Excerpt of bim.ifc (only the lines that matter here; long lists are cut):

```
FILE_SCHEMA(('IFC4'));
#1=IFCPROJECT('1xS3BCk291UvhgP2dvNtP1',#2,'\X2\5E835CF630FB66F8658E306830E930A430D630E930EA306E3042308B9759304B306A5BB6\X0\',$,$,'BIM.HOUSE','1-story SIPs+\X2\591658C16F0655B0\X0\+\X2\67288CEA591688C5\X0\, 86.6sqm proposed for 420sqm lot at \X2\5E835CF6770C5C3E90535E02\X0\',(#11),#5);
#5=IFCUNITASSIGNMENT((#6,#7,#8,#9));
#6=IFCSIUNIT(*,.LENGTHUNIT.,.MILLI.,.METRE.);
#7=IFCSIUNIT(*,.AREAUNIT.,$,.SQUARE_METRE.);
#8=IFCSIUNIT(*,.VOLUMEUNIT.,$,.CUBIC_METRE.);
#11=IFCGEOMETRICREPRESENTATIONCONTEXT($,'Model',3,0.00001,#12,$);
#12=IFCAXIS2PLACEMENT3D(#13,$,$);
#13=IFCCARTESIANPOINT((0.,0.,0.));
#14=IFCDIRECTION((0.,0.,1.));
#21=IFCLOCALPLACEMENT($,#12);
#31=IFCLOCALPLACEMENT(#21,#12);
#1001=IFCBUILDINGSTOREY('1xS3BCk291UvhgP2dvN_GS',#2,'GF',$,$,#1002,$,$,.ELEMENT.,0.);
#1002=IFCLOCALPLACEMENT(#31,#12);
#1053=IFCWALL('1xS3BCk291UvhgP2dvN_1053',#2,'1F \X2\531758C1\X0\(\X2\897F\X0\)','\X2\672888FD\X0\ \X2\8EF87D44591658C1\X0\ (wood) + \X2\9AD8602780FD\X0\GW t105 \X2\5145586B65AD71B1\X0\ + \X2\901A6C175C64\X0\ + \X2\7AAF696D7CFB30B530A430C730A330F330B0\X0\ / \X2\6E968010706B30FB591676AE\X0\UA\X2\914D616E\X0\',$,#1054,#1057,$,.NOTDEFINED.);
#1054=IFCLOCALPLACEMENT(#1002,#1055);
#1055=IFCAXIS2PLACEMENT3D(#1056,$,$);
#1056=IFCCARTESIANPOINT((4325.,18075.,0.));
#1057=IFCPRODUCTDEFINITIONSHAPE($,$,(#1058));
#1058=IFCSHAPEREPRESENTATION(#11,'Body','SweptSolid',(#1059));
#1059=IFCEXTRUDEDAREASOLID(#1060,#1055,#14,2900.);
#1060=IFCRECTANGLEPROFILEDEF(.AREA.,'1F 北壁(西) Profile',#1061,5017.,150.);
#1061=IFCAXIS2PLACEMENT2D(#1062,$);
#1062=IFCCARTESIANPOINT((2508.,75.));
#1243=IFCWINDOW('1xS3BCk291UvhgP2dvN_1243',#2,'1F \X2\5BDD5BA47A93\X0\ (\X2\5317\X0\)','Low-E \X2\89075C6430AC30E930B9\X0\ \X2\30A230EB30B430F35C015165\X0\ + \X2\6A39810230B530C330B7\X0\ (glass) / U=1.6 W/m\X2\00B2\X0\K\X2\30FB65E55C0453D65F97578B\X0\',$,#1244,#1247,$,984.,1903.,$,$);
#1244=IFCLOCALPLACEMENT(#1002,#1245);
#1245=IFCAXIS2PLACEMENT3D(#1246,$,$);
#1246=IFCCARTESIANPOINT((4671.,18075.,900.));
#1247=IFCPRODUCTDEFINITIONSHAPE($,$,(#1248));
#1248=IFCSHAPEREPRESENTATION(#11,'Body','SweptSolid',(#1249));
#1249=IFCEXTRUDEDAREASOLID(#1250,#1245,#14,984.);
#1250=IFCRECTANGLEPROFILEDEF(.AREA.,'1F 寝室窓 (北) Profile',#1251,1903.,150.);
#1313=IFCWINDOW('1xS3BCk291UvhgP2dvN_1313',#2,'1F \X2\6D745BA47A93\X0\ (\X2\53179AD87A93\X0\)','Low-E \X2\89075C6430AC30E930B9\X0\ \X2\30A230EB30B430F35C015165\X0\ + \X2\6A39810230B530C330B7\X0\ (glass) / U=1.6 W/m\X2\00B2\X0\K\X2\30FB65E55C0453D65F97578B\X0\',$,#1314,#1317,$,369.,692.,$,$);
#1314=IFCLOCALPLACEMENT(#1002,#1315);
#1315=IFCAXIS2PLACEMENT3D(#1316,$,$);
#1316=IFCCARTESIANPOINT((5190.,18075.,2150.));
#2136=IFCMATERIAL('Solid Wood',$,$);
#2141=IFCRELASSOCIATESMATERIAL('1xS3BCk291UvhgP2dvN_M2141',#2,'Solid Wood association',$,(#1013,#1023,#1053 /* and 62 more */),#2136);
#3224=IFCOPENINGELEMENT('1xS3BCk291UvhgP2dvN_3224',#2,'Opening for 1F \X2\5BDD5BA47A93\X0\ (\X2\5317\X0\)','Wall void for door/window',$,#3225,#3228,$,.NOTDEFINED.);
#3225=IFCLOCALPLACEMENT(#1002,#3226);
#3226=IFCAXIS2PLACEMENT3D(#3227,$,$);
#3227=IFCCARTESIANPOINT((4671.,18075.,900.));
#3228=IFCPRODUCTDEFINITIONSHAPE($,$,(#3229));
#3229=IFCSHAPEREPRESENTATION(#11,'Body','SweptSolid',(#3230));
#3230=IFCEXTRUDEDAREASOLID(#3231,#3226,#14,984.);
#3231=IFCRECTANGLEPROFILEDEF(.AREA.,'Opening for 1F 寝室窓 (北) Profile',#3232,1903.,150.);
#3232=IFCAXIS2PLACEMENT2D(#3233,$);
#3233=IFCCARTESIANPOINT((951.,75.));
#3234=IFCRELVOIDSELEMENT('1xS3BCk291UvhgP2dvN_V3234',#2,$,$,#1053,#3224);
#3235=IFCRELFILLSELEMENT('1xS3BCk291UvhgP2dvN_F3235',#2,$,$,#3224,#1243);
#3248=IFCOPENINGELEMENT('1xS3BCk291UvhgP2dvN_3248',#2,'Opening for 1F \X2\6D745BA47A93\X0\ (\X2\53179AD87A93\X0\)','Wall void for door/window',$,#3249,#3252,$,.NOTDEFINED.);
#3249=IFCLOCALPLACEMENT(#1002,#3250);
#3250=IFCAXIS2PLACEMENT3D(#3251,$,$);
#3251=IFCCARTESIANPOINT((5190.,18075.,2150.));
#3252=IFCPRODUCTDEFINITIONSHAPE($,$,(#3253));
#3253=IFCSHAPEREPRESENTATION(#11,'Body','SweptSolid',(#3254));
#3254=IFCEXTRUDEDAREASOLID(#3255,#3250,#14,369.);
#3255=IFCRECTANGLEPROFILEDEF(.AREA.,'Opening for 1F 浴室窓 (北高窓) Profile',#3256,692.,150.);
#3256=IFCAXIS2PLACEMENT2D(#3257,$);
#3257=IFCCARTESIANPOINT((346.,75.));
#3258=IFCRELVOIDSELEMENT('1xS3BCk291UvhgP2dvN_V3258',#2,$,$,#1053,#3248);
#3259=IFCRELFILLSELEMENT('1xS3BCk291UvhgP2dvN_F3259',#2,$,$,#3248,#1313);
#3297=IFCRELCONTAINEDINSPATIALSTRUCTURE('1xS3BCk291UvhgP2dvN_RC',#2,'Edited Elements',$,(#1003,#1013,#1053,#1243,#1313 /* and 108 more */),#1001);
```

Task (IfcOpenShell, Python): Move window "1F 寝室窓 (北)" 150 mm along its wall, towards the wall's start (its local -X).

```python
import ifcopenshell
import ifcopenshell.api.geometry
import ifcopenshell.util.placement
import ifcopenshell.util.unit

model = ifcopenshell.open("bim.ifc")
unit_scale = ifcopenshell.util.unit.calculate_unit_scale(model)

window = model.by_guid("1xS3BCk291UvhgP2dvN_1243")
opening = window.FillsVoids[0].RelatingOpeningElement
wall = opening.VoidsElements[0].RelatingBuildingElement

wall_matrix = ifcopenshell.util.placement.get_local_placement(wall.ObjectPlacement)
shift = wall_matrix[:3, 0] * -0.15 / unit_scale
before = ifcopenshell.util.placement.get_local_placement(window.ObjectPlacement)[:3, 3].copy()

# The window is not placed relative to its opening, so move both.
for product in (opening, window):
    matrix = ifcopenshell.util.placement.get_local_placement(product.ObjectPlacement)
    matrix[:3, 3] += shift
    ifcopenshell.api.geometry.edit_object_placement(model, product=product, matrix=matrix, is_si=False)

after = ifcopenshell.util.placement.get_local_placement(window.ObjectPlacement)[:3, 3]
print("window moved by", (after - before).round(3) + 0.0)

model.write("bim-out.ifc")
```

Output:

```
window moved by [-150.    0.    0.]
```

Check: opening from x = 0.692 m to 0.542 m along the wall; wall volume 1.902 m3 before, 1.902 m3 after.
